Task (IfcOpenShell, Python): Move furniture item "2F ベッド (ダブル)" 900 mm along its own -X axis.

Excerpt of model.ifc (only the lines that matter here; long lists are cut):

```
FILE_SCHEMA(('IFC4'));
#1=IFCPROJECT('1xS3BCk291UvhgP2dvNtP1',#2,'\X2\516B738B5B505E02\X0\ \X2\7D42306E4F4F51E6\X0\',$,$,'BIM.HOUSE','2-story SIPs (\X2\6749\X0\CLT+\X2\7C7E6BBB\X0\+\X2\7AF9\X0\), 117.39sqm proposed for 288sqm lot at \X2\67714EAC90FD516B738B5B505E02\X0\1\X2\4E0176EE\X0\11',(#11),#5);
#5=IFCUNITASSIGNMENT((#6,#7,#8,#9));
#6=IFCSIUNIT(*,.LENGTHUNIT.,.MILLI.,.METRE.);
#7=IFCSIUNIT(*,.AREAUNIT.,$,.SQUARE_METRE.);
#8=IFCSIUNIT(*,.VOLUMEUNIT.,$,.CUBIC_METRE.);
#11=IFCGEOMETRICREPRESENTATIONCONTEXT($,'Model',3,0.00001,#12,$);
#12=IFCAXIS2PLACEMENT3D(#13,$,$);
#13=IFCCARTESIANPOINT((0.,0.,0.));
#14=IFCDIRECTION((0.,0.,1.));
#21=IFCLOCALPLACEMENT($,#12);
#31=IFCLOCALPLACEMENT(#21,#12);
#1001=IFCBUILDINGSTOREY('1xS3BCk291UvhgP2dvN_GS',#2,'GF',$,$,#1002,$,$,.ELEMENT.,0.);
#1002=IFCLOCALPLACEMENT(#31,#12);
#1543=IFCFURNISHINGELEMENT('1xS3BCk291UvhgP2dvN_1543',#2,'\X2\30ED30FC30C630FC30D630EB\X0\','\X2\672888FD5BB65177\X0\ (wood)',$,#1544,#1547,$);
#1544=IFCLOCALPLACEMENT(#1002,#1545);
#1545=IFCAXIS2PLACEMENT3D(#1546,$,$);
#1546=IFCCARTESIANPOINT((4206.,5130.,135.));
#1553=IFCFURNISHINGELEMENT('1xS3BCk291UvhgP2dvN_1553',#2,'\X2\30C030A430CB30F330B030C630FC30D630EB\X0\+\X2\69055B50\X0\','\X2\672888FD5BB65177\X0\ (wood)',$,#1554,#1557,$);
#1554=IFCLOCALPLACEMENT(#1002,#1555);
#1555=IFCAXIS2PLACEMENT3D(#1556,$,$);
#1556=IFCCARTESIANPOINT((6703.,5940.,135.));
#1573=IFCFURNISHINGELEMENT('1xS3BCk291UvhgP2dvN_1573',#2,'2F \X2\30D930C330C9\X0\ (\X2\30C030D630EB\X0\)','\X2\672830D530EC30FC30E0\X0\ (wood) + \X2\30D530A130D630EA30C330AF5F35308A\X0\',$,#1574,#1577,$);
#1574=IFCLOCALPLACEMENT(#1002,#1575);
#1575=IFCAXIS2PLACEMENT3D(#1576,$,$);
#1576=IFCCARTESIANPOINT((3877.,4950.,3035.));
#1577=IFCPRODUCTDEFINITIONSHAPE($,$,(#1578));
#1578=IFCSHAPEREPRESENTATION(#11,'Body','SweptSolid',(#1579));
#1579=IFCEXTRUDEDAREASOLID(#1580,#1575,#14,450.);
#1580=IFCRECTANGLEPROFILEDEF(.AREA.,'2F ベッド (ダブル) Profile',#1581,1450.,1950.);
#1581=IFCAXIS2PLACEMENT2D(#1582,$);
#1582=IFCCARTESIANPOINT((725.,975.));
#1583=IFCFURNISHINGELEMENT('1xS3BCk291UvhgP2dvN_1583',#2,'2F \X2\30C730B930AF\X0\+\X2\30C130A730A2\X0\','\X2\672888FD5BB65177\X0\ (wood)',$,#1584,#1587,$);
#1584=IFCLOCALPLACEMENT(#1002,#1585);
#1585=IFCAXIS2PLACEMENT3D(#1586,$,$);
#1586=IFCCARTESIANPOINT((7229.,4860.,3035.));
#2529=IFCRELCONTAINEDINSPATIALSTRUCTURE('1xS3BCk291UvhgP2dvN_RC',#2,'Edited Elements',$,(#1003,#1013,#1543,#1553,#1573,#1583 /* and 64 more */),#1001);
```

```python
import ifcopenshell
import ifcopenshell.api.geometry
import ifcopenshell.util.placement

model = ifcopenshell.open("model.ifc")

item = model.by_guid("1xS3BCk291UvhgP2dvN_1573")
matrix = ifcopenshell.util.placement.get_local_placement(item.ObjectPlacement)
matrix[:3, 3] -= matrix[:3, 0] * 900.0
ifcopenshell.api.geometry.edit_object_placement(model, product=item, matrix=matrix, is_si=False)

print(ifcopenshell.util.placement.get_local_placement(item.ObjectPlacement).round(3) + 0.0)

model.write("model_edited.ifc")
```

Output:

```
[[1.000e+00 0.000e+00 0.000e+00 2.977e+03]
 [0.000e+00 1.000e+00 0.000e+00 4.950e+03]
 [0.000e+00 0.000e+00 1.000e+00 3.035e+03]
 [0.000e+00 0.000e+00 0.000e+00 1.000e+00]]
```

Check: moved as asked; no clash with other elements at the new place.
